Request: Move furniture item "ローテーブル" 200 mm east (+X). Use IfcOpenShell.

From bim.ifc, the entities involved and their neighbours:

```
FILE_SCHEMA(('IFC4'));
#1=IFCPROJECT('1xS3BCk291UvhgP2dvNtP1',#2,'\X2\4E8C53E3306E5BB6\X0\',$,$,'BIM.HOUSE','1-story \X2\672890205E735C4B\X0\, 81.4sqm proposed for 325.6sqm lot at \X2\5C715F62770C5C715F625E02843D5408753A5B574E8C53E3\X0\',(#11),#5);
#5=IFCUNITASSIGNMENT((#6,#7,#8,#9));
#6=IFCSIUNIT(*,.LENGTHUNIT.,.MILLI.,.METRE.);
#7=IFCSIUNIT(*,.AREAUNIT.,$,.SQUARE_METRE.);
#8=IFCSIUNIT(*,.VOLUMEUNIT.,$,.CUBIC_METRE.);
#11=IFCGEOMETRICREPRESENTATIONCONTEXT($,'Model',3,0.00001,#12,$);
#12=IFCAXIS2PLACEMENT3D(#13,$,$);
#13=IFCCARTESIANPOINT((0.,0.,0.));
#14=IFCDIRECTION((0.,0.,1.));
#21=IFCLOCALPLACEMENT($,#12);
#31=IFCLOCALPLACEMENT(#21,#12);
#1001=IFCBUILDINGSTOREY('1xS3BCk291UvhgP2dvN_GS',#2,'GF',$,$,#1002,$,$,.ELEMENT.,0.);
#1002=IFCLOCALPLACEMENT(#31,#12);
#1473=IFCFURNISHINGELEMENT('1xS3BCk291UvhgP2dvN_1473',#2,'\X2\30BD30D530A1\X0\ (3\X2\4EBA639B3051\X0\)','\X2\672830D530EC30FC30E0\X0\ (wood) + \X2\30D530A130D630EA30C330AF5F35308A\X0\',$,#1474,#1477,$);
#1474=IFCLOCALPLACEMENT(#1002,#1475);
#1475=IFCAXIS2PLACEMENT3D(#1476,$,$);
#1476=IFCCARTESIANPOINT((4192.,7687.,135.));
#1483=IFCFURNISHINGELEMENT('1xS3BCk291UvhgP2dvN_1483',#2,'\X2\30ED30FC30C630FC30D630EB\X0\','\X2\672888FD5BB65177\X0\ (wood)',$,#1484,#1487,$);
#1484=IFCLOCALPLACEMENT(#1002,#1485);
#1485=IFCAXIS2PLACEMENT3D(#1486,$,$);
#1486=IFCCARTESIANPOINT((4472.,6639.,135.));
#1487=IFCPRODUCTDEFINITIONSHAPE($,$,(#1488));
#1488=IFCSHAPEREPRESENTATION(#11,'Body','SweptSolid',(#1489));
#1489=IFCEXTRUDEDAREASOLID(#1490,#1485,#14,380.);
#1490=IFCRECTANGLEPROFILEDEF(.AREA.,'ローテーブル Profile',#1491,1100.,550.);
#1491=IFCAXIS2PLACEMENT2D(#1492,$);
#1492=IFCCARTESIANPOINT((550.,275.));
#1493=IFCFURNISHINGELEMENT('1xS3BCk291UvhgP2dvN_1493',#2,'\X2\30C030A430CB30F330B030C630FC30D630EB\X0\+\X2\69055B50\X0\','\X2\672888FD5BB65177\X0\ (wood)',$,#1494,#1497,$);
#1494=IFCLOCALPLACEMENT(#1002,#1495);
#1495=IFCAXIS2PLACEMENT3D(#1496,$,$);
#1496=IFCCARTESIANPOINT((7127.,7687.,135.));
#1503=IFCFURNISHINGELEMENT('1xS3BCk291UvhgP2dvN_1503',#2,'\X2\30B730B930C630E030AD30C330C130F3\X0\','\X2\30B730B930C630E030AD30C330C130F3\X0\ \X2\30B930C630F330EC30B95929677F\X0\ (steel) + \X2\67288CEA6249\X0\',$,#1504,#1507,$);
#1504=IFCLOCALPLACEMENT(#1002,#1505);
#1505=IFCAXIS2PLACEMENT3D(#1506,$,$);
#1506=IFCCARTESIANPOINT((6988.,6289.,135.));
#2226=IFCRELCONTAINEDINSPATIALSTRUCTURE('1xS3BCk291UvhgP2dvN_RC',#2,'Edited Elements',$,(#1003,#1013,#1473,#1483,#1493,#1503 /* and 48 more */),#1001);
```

```python
import ifcopenshell
import ifcopenshell.api.geometry
import ifcopenshell.util.placement
import ifcopenshell.util.unit

model = ifcopenshell.open("bim.ifc")
unit_scale = ifcopenshell.util.unit.calculate_unit_scale(model)

item = model.by_id(1483)
matrix = ifcopenshell.util.placement.get_local_placement(item.ObjectPlacement)
matrix[0, 3] += 0.2 / unit_scale
ifcopenshell.api.geometry.edit_object_placement(model, product=item, matrix=matrix, is_si=False)

print(ifcopenshell.util.placement.get_local_placement(item.ObjectPlacement).round(3) + 0.0)

model.write("bim-out.ifc")
```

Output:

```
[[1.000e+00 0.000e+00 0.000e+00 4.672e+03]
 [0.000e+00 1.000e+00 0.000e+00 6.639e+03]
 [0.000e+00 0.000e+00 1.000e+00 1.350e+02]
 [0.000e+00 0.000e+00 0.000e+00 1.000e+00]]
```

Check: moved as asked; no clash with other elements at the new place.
